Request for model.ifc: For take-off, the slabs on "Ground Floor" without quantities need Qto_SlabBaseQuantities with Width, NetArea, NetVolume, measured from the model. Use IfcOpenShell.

First a look at what the model holds.

```python
import ifcopenshell
import ifcopenshell.util.element
import ifcopenshell.util.unit

model = ifcopenshell.open("model.ifc")
print(model.schema)
for unit_type in ("LENGTHUNIT", "AREAUNIT", "VOLUMEUNIT"):
    print(unit_type, ifcopenshell.util.unit.calculate_unit_scale(model, unit_type))
storey = next(s for s in model.by_type("IfcBuildingStorey") if s.Name == "Ground Floor")
slabs = [e for e in ifcopenshell.util.element.get_decomposition(storey) if e.is_a("IfcSlab")]
for e in sorted(slabs, key=lambda e: e.id()):
    print(e.id(), e.is_a(), e.Name, list(ifcopenshell.util.element.get_psets(e, qtos_only=True)), sep=" | ")
```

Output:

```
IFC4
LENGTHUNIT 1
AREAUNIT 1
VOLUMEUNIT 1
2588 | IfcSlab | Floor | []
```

```python
import ifcopenshell
import ifcopenshell.api.pset
import ifcopenshell.geom
import ifcopenshell.util.element
import ifcopenshell.util.shape
import ifcopenshell.util.unit

model = ifcopenshell.open("model.ifc")
unit_scale = ifcopenshell.util.unit.calculate_unit_scale(model)
area_scale = ifcopenshell.util.unit.calculate_unit_scale(model, "AREAUNIT")
volume_scale = ifcopenshell.util.unit.calculate_unit_scale(model, "VOLUMEUNIT")
settings = ifcopenshell.geom.settings()

storey = next(s for s in model.by_type("IfcBuildingStorey") if s.Name == "Ground Floor")
slabs = [e for e in ifcopenshell.util.element.get_decomposition(storey) if e.is_a("IfcSlab")]

for e in sorted(slabs, key=lambda e: e.id()):
    if ifcopenshell.util.element.get_psets(e, qtos_only=True, should_inherit=False):
        continue
    # Geometry comes back in metres, in the element's own axes.
    shape = ifcopenshell.geom.create_shape(settings, e)
    values = {
        "Width": ifcopenshell.util.shape.get_z(shape.geometry) / unit_scale,
        "NetArea": ifcopenshell.util.shape.get_footprint_area(shape.geometry) / area_scale,
        "NetVolume": ifcopenshell.util.shape.get_volume(shape.geometry) / volume_scale,
    }
    qto = ifcopenshell.api.pset.add_qto(model, product=e, name="Qto_SlabBaseQuantities")
    ifcopenshell.api.pset.edit_qto(model, qto=qto, properties=values)
    print(e.id(), {k: round(v, 3) for k, v in values.items()})

model.write("model-out.ifc")
```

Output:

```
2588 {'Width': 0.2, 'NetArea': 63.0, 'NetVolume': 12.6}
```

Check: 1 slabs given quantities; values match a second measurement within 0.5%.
